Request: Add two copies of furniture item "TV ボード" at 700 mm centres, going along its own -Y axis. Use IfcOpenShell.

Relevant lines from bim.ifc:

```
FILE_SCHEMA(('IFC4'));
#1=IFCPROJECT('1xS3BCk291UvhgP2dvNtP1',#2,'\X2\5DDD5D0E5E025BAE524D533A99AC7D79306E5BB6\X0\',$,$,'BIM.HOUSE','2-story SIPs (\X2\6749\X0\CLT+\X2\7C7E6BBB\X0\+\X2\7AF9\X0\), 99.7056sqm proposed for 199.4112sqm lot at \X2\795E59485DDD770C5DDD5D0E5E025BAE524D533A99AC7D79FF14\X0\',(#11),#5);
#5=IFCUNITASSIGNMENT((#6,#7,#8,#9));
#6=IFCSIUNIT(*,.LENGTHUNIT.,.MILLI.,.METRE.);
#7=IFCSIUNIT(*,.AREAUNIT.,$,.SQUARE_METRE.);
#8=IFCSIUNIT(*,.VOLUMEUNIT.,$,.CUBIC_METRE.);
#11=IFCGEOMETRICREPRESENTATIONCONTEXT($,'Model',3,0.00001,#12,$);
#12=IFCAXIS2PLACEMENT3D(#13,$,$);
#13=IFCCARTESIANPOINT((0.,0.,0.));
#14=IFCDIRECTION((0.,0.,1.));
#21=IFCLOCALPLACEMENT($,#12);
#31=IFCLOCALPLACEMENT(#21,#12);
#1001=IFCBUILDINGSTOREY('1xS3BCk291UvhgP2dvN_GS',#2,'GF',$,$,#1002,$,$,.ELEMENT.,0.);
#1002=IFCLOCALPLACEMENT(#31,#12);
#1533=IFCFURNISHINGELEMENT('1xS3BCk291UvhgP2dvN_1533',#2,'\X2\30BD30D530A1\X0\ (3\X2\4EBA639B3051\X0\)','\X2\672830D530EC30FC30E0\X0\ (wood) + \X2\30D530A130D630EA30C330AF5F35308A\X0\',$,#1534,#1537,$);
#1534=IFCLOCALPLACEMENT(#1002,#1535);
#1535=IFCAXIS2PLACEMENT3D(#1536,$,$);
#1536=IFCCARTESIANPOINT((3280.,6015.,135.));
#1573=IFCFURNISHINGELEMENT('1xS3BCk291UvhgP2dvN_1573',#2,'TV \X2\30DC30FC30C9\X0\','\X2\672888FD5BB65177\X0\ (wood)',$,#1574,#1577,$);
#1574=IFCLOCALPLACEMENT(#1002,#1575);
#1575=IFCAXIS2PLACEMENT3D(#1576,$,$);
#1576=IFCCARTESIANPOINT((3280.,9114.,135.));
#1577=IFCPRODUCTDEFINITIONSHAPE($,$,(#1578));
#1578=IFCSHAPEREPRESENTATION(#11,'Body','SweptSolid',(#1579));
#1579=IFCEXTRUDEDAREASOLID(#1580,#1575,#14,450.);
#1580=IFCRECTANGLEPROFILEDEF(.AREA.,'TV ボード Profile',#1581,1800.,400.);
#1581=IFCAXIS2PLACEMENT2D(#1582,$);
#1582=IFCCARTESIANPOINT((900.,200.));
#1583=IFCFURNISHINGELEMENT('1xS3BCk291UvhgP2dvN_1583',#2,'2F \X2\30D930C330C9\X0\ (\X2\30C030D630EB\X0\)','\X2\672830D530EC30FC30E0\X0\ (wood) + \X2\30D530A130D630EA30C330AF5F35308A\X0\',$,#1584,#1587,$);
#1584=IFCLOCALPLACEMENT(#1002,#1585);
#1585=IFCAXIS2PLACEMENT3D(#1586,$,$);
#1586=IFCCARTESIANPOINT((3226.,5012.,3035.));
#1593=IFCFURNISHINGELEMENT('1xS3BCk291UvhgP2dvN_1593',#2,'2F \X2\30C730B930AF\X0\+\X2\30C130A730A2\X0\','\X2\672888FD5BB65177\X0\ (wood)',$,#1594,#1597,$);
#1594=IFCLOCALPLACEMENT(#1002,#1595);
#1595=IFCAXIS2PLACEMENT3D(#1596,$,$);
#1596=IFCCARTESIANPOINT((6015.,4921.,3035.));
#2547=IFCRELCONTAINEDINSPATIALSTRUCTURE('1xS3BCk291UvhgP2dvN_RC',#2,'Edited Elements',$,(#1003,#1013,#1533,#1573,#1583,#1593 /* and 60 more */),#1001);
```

```python
import ifcopenshell
import ifcopenshell.api.geometry
import ifcopenshell.api.root
import ifcopenshell.util.element
import ifcopenshell.util.placement

model = ifcopenshell.open("bim.ifc")


def reuse_history(source, copy):
    """copy_class also copies each property set's owner history, people and application; keep the originals."""
    for rel in copy.IsDefinedBy:
        if rel.is_a("IfcRelDefinesByProperties") and (history := rel.RelatingPropertyDefinition.OwnerHistory):
            rel.RelatingPropertyDefinition.OwnerHistory = source.OwnerHistory
            ifcopenshell.util.element.remove_deep2(model, history)


source = model.by_guid("1xS3BCk291UvhgP2dvN_1573")
base = ifcopenshell.util.placement.get_local_placement(source.ObjectPlacement)
step = -base[:3, 1] * 700.0

for i in range(1, 3):
    copy = ifcopenshell.api.root.copy_class(model, product=source)
    copy.Representation = ifcopenshell.util.element.copy_deep(
        model, source.Representation, exclude=["IfcGeometricRepresentationContext", "IfcRepresentationMap"]
    )
    reuse_history(source, copy)
    matrix = base.copy()
    matrix[:3, 3] += i * step
    print("added at", matrix[:3, 3].round(3) + 0.0)
    ifcopenshell.api.geometry.edit_object_placement(model, product=copy, matrix=matrix, is_si=False)

model.write("bim_v2.ifc")
```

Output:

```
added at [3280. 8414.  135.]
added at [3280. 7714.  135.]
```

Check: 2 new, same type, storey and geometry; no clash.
